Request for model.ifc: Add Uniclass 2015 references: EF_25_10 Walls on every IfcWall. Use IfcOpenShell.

First a look at what the model holds.

```python
import ifcopenshell

model = ifcopenshell.open("model.ifc")
print(model.schema)
print("classifications:", [c.Name for c in model.by_type("IfcClassification")])
for ifc_class in ("IfcDoor", "IfcRoof", "IfcStair", "IfcWall", "IfcWindow"):
    print(ifc_class, len(model.by_type(ifc_class)))
```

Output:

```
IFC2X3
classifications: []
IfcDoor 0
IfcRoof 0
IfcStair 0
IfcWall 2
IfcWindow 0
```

```python
import ifcopenshell
import ifcopenshell.api.classification

model = ifcopenshell.open("model.ifc")

# IFC2X3 requires Source and Edition and has no link from the project to the system.
system = model.create_entity("IfcClassification", Source="NBS", Edition="2015", Name="Uniclass 2015")

codes = {
    "IfcWall": ("EF_25_10", "Walls"),
}
for ifc_class, (code, name) in codes.items():
    products = model.by_type(ifc_class)
    ifcopenshell.api.classification.add_reference(
        model, products=products, classification=system, identification=code, name=name
    )
    print(code, len(products))

model.write("model_updated.ifc")
```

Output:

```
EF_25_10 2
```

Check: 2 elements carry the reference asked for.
